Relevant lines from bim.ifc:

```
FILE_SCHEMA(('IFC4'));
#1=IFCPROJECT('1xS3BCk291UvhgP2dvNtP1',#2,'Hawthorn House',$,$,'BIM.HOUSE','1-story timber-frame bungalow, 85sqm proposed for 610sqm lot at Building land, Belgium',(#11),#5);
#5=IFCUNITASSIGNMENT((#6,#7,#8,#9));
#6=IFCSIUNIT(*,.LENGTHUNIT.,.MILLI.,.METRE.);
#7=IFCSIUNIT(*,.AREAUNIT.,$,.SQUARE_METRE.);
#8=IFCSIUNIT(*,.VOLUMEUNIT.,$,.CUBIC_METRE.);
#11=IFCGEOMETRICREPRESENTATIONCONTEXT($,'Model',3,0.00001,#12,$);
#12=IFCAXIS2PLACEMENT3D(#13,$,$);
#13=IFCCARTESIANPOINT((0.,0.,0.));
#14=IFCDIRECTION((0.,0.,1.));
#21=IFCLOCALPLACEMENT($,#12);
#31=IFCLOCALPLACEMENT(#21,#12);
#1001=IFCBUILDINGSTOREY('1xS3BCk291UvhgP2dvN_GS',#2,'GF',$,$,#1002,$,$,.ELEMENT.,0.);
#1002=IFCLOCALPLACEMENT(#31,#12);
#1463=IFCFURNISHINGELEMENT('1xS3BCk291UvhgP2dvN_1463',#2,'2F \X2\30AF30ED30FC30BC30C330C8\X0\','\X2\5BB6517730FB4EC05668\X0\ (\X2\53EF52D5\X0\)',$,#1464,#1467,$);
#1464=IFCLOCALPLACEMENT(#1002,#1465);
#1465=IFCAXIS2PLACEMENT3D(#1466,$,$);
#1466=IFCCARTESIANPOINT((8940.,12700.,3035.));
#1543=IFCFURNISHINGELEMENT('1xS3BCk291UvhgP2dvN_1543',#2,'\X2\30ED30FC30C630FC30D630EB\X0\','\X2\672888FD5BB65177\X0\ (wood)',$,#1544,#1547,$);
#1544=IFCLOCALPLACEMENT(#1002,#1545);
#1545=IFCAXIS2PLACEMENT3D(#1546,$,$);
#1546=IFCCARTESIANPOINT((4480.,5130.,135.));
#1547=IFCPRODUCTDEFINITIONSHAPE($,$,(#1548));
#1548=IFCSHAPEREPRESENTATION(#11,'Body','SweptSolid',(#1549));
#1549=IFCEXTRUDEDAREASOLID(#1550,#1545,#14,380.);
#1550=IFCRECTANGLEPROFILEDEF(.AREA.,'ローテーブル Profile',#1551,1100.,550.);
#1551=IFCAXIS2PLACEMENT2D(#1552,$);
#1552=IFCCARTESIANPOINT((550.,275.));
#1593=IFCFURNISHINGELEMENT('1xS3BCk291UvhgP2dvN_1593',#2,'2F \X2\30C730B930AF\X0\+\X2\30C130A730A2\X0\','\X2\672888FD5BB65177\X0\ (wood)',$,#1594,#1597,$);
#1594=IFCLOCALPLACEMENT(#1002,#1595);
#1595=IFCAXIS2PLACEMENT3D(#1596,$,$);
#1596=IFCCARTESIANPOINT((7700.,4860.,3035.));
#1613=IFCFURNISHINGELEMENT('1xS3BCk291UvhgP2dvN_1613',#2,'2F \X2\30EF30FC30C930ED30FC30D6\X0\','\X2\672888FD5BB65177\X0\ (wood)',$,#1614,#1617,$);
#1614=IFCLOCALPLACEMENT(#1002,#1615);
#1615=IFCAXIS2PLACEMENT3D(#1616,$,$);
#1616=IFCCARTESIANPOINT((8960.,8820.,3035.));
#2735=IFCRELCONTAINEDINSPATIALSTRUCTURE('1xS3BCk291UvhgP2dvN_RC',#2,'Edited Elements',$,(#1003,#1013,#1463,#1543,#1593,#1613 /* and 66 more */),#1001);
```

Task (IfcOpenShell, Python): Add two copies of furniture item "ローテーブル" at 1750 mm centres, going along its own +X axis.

```python
import ifcopenshell
import ifcopenshell.api.geometry
import ifcopenshell.api.root
import ifcopenshell.util.element
import ifcopenshell.util.placement

model = ifcopenshell.open("bim.ifc")


def reuse_history(source, copy):
    """copy_class also copies each property set's owner history, people and application; keep the originals."""
    for rel in copy.IsDefinedBy:
        if rel.is_a("IfcRelDefinesByProperties") and (history := rel.RelatingPropertyDefinition.OwnerHistory):
            rel.RelatingPropertyDefinition.OwnerHistory = source.OwnerHistory
            ifcopenshell.util.element.remove_deep2(model, history)


source = model.by_id(1543)
base = ifcopenshell.util.placement.get_local_placement(source.ObjectPlacement)
step = base[:3, 0] * 1750.0

for i in range(1, 3):
    copy = ifcopenshell.api.root.copy_class(model, product=source)
    copy.Representation = ifcopenshell.util.element.copy_deep(
        model, source.Representation, exclude=["IfcGeometricRepresentationContext", "IfcRepresentationMap"]
    )
    reuse_history(source, copy)
    matrix = base.copy()
    matrix[:3, 3] += i * step
    print("added at", matrix[:3, 3].round(3) + 0.0)
    ifcopenshell.api.geometry.edit_object_placement(model, product=copy, matrix=matrix, is_si=False)

model.write("bim_edited.ifc")
```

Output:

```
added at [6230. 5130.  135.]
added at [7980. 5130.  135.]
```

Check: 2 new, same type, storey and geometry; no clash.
